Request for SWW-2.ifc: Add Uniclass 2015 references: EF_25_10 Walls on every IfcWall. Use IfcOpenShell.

First a look at what the model holds.

```python
import ifcopenshell

model = ifcopenshell.open("SWW-2.ifc")
print(model.schema)
print("classifications:", [c.Name for c in model.by_type("IfcClassification")])
for ifc_class in ("IfcDoor", "IfcRoof", "IfcStair", "IfcWall", "IfcWindow"):
    print(ifc_class, len(model.by_type(ifc_class)))
```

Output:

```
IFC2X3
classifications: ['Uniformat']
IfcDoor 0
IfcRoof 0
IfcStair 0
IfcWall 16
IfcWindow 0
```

```python
import ifcopenshell
import ifcopenshell.api.classification

model = ifcopenshell.open("SWW-2.ifc")

# IFC2X3 requires Source and Edition and has no link from the project to the system.
system = model.create_entity("IfcClassification", Source="NBS", Edition="2015", Name="Uniclass 2015")

codes = {
    "IfcWall": ("EF_25_10", "Walls"),
}
for ifc_class, (code, name) in codes.items():
    products = model.by_type(ifc_class)
    ifcopenshell.api.classification.add_reference(
        model, products=products, classification=system, identification=code, name=name
    )
    print(code, len(products))

model.write("SWW-2-out.ifc")
```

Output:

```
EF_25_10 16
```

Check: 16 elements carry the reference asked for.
